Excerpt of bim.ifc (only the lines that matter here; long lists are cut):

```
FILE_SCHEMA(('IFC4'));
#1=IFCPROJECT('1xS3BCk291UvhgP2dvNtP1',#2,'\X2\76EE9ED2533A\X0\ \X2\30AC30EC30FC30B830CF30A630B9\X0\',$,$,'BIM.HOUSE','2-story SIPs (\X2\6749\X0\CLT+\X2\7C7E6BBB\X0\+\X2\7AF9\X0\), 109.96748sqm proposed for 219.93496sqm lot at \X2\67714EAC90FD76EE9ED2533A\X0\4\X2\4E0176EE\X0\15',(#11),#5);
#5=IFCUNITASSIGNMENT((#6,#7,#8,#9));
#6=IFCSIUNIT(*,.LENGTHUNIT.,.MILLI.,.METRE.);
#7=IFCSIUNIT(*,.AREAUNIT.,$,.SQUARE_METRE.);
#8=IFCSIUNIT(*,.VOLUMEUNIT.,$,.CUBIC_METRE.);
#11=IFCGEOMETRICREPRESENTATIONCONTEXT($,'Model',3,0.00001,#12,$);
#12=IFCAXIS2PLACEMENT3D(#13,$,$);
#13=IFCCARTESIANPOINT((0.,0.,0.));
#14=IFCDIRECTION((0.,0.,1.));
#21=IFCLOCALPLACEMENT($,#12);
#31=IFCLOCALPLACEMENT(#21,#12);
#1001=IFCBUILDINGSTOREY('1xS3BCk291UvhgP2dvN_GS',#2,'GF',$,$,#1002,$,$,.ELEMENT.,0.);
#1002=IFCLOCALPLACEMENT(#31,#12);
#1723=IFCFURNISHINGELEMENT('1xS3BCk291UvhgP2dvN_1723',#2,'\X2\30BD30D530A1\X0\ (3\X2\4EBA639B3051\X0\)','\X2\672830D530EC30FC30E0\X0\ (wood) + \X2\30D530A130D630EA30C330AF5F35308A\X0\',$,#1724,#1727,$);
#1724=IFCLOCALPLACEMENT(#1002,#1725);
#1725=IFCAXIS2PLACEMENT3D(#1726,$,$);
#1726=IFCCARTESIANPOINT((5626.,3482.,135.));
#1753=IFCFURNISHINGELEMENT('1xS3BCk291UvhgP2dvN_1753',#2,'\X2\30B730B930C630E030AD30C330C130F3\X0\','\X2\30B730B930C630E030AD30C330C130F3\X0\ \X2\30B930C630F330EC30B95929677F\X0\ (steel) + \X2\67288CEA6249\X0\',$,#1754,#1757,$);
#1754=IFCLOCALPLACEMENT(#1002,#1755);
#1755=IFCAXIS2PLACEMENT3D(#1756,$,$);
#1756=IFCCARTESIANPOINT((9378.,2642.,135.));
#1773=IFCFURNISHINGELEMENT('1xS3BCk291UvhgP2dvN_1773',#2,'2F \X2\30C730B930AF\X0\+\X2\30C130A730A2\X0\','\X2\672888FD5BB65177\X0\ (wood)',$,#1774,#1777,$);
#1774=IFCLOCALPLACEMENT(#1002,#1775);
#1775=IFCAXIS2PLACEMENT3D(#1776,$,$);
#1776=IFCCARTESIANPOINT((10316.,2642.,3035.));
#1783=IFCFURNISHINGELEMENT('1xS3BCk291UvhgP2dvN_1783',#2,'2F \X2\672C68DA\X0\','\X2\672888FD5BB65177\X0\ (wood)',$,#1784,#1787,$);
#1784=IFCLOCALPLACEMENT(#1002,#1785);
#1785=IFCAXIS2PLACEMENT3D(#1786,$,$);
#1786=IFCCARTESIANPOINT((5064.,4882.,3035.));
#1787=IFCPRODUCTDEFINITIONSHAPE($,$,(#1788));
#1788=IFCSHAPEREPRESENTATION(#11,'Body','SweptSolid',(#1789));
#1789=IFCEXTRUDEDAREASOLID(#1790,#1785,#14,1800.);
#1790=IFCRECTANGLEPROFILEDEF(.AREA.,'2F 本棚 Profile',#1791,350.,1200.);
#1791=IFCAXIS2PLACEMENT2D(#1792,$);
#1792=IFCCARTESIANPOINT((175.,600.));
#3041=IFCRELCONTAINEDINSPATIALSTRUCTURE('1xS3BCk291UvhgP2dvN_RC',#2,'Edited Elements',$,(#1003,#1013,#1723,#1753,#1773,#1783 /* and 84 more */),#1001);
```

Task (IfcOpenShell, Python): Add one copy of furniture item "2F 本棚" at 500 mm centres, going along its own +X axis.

```python
import ifcopenshell
import ifcopenshell.api.geometry
import ifcopenshell.api.root
import ifcopenshell.util.element
import ifcopenshell.util.placement
import ifcopenshell.util.unit

model = ifcopenshell.open("bim.ifc")
unit_scale = ifcopenshell.util.unit.calculate_unit_scale(model)


def reuse_history(source, copy):
    """copy_class also copies each property set's owner history, people and application; keep the originals."""
    for rel in copy.IsDefinedBy:
        if rel.is_a("IfcRelDefinesByProperties") and (history := rel.RelatingPropertyDefinition.OwnerHistory):
            rel.RelatingPropertyDefinition.OwnerHistory = source.OwnerHistory
            ifcopenshell.util.element.remove_deep2(model, history)


source = model.by_guid("1xS3BCk291UvhgP2dvN_1783")
base = ifcopenshell.util.placement.get_local_placement(source.ObjectPlacement)
step = base[:3, 0] * 0.5 / unit_scale

for i in range(1, 2):
    copy = ifcopenshell.api.root.copy_class(model, product=source)
    copy.Representation = ifcopenshell.util.element.copy_deep(
        model, source.Representation, exclude=["IfcGeometricRepresentationContext", "IfcRepresentationMap"]
    )
    reuse_history(source, copy)
    matrix = base.copy()
    matrix[:3, 3] += i * step
    print("added at", matrix[:3, 3].round(3) + 0.0)
    ifcopenshell.api.geometry.edit_object_placement(model, product=copy, matrix=matrix, is_si=False)

model.write("bim_updated.ifc")
```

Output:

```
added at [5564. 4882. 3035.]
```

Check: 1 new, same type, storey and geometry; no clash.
